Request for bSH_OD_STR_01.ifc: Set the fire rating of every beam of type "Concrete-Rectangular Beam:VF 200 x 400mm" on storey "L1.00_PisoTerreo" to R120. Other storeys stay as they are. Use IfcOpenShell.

First a look at what the model holds.

```python
import ifcopenshell
import ifcopenshell.util.element

model = ifcopenshell.open("bSH_OD_STR_01.ifc")
print(model.schema)
storey = next(s for s in model.by_type("IfcBuildingStorey") if s.Name == "L1.00_PisoTerreo")
beams = [e for e in ifcopenshell.util.element.get_decomposition(storey) if e.is_a("IfcBeam")]
seen = {}
for e in beams:
    element_type = ifcopenshell.util.element.get_type(e)
    key = (element_type.Name if element_type != e and element_type else None, ifcopenshell.util.element.get_pset(e, "Pset_BeamCommon", "FireRating"))
    seen[key] = seen.get(key, 0) + 1
for (name, value), count in sorted(seen.items(), key=str):
    print(count, "x", name, "|", value)
```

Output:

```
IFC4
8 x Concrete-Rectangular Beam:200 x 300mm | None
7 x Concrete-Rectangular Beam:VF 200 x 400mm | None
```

```python
import ifcopenshell
import ifcopenshell.api.pset
import ifcopenshell.util.element

model = ifcopenshell.open("bSH_OD_STR_01.ifc")

storey = next(s for s in model.by_type("IfcBuildingStorey") if s.Name == "L1.00_PisoTerreo")
beams = [e for e in ifcopenshell.util.element.get_decomposition(storey) if e.is_a("IfcBeam")]

count = 0
for e in beams:
    element_type = ifcopenshell.util.element.get_type(e)
    if element_type in (None, e) or element_type.Name != "Concrete-Rectangular Beam:VF 200 x 400mm":
        continue
    # add_pset returns the element's existing set when there is one.
    pset = ifcopenshell.api.pset.add_pset(model, product=e, name="Pset_BeamCommon")
    ifcopenshell.api.pset.edit_pset(model, pset=pset, properties={"FireRating": "R120"})
    count += 1

print(count, "beams updated")

model.write("bSH_OD_STR_01_rev.ifc")
```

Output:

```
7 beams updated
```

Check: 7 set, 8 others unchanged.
